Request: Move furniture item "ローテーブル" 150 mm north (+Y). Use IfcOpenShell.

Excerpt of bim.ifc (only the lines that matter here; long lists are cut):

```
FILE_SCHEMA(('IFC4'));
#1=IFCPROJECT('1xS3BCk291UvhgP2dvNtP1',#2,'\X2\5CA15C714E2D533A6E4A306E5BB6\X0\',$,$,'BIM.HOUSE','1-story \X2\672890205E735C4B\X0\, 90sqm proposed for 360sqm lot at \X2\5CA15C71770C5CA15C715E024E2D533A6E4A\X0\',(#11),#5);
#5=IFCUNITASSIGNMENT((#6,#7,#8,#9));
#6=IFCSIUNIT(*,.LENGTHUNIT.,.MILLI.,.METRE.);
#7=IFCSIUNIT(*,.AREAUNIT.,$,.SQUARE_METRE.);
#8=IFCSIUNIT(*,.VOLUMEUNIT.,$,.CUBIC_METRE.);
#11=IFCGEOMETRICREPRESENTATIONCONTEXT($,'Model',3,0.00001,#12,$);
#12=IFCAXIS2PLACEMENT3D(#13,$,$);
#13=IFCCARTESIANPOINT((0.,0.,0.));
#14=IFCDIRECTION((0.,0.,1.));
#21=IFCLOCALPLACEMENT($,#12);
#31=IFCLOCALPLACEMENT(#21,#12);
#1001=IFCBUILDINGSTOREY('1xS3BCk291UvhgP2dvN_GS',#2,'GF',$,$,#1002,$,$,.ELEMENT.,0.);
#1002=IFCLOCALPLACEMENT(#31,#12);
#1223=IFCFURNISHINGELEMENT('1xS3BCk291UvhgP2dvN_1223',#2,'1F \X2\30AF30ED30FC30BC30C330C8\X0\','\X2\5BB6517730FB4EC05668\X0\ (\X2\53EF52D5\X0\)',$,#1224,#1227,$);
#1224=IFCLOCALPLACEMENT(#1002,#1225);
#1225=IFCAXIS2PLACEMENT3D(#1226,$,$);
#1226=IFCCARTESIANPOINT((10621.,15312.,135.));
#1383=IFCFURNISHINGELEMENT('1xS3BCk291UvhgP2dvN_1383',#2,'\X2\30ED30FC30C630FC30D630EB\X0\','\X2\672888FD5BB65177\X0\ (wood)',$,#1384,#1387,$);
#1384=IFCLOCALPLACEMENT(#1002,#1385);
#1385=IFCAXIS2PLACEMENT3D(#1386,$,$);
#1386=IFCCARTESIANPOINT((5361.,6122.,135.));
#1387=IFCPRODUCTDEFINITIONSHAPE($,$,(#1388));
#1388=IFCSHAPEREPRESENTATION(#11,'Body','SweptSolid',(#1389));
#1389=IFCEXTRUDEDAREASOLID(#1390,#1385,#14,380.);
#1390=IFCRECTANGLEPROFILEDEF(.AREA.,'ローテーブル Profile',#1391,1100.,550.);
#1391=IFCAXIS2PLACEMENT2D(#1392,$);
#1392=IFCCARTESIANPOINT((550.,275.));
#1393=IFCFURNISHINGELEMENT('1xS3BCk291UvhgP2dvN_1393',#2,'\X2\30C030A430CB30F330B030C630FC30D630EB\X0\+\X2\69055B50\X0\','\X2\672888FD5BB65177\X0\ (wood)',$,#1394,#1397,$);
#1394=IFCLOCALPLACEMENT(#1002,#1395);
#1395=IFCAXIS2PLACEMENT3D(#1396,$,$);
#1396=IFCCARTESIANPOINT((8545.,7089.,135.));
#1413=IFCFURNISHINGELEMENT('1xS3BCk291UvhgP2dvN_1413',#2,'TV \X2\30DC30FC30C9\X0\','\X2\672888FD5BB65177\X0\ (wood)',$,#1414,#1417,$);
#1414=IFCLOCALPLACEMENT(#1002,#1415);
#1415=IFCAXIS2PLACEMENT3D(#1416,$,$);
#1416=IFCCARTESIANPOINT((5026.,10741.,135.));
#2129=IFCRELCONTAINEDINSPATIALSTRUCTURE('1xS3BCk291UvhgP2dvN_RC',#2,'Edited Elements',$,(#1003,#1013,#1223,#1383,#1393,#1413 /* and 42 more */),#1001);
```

```python
import ifcopenshell
import ifcopenshell.api.geometry
import ifcopenshell.util.placement
import ifcopenshell.util.unit

model = ifcopenshell.open("bim.ifc")
unit_scale = ifcopenshell.util.unit.calculate_unit_scale(model)

item = model.by_guid("1xS3BCk291UvhgP2dvN_1383")
matrix = ifcopenshell.util.placement.get_local_placement(item.ObjectPlacement)
matrix[1, 3] += 0.15 / unit_scale
ifcopenshell.api.geometry.edit_object_placement(model, product=item, matrix=matrix, is_si=False)

print(ifcopenshell.util.placement.get_local_placement(item.ObjectPlacement).round(3) + 0.0)

model.write("bim_rev.ifc")
```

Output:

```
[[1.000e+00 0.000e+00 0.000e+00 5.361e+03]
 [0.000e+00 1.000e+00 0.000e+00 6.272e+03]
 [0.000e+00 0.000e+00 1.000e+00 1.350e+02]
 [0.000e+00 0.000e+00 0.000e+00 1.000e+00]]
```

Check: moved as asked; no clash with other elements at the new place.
